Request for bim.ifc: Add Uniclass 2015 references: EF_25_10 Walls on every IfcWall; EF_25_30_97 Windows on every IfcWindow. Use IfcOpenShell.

First a look at what the model holds.

```python
import ifcopenshell

model = ifcopenshell.open("bim.ifc")
print(model.schema)
print("classifications:", [c.Name for c in model.by_type("IfcClassification")])
for ifc_class in ("IfcDoor", "IfcRoof", "IfcStair", "IfcWall", "IfcWindow"):
    print(ifc_class, len(model.by_type(ifc_class)))
```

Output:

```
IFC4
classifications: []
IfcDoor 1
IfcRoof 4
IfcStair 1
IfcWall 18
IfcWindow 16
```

```python
import ifcopenshell
import ifcopenshell.api.classification

model = ifcopenshell.open("bim.ifc")

system = ifcopenshell.api.classification.add_classification(model, classification="Uniclass 2015")

codes = {
    "IfcWall": ("EF_25_10", "Walls"),
    "IfcWindow": ("EF_25_30_97", "Windows"),
}
for ifc_class, (code, name) in codes.items():
    products = model.by_type(ifc_class)
    ifcopenshell.api.classification.add_reference(
        model, products=products, classification=system, identification=code, name=name
    )
    print(code, len(products))

model.write("bim_rev.ifc")
```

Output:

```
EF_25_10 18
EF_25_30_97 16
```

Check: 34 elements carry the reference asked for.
